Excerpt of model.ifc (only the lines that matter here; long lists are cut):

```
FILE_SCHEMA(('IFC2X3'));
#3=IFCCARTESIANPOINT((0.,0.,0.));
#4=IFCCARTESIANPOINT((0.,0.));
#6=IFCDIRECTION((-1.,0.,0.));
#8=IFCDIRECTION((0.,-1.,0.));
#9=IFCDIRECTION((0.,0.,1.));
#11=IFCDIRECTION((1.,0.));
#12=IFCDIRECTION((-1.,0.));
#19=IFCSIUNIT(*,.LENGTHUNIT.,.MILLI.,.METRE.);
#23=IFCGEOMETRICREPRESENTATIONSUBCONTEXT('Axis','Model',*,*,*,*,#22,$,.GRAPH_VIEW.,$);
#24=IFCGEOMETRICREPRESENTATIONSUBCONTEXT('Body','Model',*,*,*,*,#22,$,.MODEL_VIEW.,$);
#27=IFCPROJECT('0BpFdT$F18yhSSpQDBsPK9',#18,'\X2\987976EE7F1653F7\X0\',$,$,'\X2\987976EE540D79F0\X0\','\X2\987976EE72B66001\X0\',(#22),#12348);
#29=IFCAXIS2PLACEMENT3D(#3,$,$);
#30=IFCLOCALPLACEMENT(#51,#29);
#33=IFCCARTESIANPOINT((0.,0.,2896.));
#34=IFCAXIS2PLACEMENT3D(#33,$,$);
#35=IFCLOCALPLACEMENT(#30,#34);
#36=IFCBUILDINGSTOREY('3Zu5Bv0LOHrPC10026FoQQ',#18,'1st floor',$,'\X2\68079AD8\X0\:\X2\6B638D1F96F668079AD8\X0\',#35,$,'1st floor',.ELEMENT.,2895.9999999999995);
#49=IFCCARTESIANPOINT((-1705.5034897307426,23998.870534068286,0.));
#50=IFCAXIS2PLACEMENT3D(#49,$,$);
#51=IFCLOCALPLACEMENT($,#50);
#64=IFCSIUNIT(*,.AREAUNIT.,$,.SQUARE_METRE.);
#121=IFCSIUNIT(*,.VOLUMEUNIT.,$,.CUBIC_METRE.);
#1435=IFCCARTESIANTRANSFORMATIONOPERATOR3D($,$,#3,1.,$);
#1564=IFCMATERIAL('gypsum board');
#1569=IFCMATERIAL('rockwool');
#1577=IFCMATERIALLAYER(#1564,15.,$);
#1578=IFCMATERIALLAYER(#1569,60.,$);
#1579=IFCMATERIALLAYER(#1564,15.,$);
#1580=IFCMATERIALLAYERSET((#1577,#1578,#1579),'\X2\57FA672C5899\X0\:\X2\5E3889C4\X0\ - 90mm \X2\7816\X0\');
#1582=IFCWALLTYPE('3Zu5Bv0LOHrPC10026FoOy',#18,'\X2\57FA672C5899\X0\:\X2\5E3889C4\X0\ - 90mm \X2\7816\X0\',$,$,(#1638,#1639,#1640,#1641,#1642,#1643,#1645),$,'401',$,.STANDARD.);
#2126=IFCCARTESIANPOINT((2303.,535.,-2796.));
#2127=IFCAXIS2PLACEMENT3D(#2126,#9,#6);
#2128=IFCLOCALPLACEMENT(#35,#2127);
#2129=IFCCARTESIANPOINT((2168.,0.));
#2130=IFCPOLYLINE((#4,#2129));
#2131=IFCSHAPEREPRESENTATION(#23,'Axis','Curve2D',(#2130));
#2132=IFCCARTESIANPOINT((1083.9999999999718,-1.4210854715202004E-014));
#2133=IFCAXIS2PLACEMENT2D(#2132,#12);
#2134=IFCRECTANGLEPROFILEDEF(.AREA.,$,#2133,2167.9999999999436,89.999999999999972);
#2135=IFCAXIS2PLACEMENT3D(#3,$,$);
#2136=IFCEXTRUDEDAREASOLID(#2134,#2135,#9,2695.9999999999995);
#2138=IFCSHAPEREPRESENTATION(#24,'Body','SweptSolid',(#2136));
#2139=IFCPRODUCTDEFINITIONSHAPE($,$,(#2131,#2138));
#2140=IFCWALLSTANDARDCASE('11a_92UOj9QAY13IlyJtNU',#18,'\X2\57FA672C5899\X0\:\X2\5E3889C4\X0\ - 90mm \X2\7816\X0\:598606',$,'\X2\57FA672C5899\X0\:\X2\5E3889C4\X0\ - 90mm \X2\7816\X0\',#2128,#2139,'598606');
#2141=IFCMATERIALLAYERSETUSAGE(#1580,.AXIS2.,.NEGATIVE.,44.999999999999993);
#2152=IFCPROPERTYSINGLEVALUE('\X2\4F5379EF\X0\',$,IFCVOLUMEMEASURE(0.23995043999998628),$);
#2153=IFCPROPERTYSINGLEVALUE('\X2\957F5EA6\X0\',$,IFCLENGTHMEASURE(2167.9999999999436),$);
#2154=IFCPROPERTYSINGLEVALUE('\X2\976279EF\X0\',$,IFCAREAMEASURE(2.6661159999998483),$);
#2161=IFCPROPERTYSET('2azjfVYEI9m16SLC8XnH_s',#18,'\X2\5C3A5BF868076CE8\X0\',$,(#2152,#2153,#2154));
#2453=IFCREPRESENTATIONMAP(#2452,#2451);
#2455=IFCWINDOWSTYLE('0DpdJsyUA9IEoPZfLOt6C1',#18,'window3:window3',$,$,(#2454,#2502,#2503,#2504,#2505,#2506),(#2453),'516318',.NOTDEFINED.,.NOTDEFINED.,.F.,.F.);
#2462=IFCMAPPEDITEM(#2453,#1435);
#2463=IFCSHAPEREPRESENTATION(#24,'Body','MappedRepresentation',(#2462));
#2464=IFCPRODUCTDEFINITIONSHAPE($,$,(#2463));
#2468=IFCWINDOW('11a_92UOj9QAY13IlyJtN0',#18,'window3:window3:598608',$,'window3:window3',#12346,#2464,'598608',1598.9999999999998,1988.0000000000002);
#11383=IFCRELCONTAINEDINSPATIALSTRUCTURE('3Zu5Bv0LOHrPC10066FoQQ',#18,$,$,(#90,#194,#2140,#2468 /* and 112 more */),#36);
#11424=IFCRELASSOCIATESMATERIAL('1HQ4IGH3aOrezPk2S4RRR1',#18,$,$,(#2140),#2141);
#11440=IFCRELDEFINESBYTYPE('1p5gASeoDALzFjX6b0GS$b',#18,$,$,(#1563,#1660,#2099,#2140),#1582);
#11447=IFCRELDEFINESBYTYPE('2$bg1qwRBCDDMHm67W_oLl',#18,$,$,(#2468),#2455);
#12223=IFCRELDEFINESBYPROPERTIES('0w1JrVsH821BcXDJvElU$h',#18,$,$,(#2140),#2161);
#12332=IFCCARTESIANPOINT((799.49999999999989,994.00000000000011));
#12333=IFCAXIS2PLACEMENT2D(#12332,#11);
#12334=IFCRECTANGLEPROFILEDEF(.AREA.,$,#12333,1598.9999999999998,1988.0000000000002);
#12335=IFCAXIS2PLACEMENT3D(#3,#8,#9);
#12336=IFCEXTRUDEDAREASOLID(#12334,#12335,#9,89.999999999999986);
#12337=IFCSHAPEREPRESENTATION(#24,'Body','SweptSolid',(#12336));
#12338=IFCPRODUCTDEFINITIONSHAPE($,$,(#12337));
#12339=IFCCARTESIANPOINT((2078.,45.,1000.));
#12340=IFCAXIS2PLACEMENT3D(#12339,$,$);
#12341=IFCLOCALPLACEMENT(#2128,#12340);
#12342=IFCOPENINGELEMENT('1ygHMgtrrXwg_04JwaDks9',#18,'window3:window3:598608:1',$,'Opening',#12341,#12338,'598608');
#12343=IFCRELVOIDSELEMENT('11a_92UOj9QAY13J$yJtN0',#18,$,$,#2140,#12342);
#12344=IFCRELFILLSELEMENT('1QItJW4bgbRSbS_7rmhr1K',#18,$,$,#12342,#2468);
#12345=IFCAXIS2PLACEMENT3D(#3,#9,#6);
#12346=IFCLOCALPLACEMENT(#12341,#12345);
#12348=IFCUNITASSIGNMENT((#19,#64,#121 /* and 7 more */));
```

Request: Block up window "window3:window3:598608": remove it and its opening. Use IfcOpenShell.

```python
import ifcopenshell
import ifcopenshell.api.feature
import ifcopenshell.api.pset
import ifcopenshell.api.root
import ifcopenshell.geom
import ifcopenshell.util.element
import ifcopenshell.util.shape
import ifcopenshell.util.unit

model = ifcopenshell.open("model.ifc")
area_scale = ifcopenshell.util.unit.calculate_unit_scale(model, "AREAUNIT")
volume_scale = ifcopenshell.util.unit.calculate_unit_scale(model, "VOLUMEUNIT")
settings = ifcopenshell.geom.settings()


def volume(element):
    """Net volume in cubic metres, openings subtracted."""
    shape = ifcopenshell.geom.create_shape(settings, element)
    return ifcopenshell.util.shape.get_volume(shape.geometry)


window = model.by_id(2468)
opening = window.FillsVoids[0].RelatingOpeningElement
wall = opening.VoidsElements[0].RelatingBuildingElement
before = volume(wall)

ifcopenshell.api.root.remove_product(model, product=window)
ifcopenshell.api.feature.remove_feature(model, feature=opening)

after = volume(wall)
thickness = 0.09  # wall thickness in metres

# Update the wall's stored quantities.
pset = model.by_id(ifcopenshell.util.element.get_pset(wall, "尺寸标注", should_inherit=False)["id"])
ifcopenshell.api.pset.edit_pset(model, pset=pset, properties={
    "体积": model.create_entity("IfcVolumeMeasure", after / volume_scale),
    "面积": model.create_entity("IfcAreaMeasure", after / thickness / area_scale),
})

print(f"wall volume {before:.3f} -> {after:.3f} m3")

model.write("model_edited.ifc")
```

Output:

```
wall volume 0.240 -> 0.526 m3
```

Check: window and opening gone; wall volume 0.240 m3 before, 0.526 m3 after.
